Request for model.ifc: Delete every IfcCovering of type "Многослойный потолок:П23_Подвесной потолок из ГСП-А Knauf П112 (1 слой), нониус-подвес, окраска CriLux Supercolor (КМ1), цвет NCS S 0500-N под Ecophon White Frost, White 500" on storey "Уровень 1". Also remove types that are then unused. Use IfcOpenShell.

First a look at what the model holds.

```python
import ifcopenshell
import ifcopenshell.util.element

model = ifcopenshell.open("model.ifc")
print(model.schema)
storey = next(s for s in model.by_type("IfcBuildingStorey") if s.Name == "Уровень 1")
coverings = [e for e in ifcopenshell.util.element.get_decomposition(storey) if e.is_a("IfcCovering")]
seen = {}
for e in coverings:
    element_type = ifcopenshell.util.element.get_type(e)
    name = element_type.Name if element_type not in (None, e) else None
    seen[name] = seen.get(name, 0) + 1
for name, count in sorted(seen.items(), key=str):
    print(count, "x", name)
```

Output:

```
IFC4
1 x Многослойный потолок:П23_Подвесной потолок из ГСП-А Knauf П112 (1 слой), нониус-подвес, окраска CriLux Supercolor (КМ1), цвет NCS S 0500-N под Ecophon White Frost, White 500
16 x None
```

```python
import ifcopenshell
import ifcopenshell.api.root
import ifcopenshell.util.element

model = ifcopenshell.open("model.ifc")

storey = next(s for s in model.by_type("IfcBuildingStorey") if s.Name == "Уровень 1")
coverings = [e for e in ifcopenshell.util.element.get_decomposition(storey) if e.is_a("IfcCovering")]
targets = [e for e in coverings if (t := ifcopenshell.util.element.get_type(e)) not in (None, e) and t.Name == "Многослойный потолок:П23_Подвесной потолок из ГСП-А Knauf П112 (1 слой), нониус-подвес, окраска CriLux Supercolor (КМ1), цвет NCS S 0500-N под Ecophon White Frost, White 500"]
types = {ifcopenshell.util.element.get_type(e) for e in targets} - {None, *targets}

for e in targets:
    ifcopenshell.api.root.remove_product(model, product=e)
print(len(targets), "removed")

unused = [t for t in types if not ifcopenshell.util.element.get_types(t)]
for t in unused:
    ifcopenshell.api.root.remove_product(model, product=t)
print(len(unused), "unused types removed")

model.write("model-out.ifc")
```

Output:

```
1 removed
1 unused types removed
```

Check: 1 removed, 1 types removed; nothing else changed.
